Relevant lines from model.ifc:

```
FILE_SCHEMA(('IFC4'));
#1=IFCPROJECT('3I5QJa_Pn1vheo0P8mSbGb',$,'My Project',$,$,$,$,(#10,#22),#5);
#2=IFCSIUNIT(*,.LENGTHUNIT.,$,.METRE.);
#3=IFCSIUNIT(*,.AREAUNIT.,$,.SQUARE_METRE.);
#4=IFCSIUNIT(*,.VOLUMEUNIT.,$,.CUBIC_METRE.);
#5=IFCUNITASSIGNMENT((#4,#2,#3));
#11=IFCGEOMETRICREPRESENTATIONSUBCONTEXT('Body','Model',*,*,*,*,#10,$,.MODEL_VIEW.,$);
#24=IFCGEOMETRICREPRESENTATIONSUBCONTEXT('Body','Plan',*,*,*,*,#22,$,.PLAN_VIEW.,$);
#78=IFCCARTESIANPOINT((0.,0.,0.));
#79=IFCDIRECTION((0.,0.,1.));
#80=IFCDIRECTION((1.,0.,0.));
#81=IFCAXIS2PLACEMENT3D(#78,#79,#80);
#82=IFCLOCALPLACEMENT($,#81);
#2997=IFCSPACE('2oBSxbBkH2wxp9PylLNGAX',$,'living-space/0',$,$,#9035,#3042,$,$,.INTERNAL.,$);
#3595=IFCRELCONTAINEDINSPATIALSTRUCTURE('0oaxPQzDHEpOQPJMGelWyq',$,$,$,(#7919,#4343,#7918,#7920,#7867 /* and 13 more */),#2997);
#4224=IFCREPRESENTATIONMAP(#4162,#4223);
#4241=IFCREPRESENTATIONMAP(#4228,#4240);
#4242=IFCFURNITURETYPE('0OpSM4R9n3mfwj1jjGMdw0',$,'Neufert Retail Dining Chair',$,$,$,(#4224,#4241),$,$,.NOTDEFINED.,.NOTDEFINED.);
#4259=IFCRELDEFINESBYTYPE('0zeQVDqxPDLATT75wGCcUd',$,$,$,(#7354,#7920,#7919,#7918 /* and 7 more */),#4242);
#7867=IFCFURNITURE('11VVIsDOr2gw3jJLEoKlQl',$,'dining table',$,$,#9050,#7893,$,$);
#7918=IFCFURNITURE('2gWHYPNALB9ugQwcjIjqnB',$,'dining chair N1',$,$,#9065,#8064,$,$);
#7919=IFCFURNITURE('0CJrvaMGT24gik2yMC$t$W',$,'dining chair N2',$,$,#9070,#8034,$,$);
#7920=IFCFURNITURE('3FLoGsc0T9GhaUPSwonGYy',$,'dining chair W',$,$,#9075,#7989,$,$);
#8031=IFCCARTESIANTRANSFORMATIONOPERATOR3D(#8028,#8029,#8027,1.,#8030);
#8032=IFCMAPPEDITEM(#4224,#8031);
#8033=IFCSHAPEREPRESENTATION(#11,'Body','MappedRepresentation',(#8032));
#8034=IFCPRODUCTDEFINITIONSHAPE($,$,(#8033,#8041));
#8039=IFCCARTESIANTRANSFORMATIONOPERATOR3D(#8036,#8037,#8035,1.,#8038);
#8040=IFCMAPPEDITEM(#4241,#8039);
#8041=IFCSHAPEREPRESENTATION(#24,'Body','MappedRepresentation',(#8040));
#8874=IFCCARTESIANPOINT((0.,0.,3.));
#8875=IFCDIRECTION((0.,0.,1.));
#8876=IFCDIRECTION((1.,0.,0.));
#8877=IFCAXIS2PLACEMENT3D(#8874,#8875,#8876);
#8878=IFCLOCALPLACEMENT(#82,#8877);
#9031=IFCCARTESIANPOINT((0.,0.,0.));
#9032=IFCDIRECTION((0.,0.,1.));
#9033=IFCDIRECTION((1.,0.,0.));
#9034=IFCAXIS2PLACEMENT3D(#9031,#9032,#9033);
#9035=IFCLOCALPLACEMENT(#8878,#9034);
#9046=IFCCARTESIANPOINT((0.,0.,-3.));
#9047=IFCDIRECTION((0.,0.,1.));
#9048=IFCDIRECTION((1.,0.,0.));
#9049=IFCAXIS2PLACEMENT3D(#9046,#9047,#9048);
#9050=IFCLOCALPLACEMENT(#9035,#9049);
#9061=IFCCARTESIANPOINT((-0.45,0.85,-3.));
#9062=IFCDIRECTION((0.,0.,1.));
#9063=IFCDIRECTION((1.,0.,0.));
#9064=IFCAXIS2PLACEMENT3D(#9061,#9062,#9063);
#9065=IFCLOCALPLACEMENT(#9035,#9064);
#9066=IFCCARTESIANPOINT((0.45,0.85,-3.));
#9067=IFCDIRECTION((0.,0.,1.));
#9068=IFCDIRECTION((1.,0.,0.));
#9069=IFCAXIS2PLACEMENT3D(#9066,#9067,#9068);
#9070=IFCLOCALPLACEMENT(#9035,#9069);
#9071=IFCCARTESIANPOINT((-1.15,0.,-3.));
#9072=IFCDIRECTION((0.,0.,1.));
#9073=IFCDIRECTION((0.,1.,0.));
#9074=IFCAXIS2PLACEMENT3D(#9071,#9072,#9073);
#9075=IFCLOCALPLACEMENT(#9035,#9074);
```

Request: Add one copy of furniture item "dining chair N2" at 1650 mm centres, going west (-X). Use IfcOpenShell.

```python
import numpy as np
import ifcopenshell
import ifcopenshell.api.geometry
import ifcopenshell.api.root
import ifcopenshell.util.element
import ifcopenshell.util.placement
import ifcopenshell.util.unit

model = ifcopenshell.open("model.ifc")
unit_scale = ifcopenshell.util.unit.calculate_unit_scale(model)

source = model.by_id(7919)
base = ifcopenshell.util.placement.get_local_placement(source.ObjectPlacement)
step = np.array([-1.0, 0.0, 0.0]) * 1.65 / unit_scale

for i in range(1, 2):
    copy = ifcopenshell.api.root.copy_class(model, product=source)
    copy.Representation = ifcopenshell.util.element.copy_deep(
        model, source.Representation, exclude=["IfcGeometricRepresentationContext", "IfcRepresentationMap"]
    )
    matrix = base.copy()
    matrix[:3, 3] += i * step
    print("added at", matrix[:3, 3].round(3) + 0.0)
    ifcopenshell.api.geometry.edit_object_placement(model, product=copy, matrix=matrix, is_si=False)

model.write("model_edited.ifc")
```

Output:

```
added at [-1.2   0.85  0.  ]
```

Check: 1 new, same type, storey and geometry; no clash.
